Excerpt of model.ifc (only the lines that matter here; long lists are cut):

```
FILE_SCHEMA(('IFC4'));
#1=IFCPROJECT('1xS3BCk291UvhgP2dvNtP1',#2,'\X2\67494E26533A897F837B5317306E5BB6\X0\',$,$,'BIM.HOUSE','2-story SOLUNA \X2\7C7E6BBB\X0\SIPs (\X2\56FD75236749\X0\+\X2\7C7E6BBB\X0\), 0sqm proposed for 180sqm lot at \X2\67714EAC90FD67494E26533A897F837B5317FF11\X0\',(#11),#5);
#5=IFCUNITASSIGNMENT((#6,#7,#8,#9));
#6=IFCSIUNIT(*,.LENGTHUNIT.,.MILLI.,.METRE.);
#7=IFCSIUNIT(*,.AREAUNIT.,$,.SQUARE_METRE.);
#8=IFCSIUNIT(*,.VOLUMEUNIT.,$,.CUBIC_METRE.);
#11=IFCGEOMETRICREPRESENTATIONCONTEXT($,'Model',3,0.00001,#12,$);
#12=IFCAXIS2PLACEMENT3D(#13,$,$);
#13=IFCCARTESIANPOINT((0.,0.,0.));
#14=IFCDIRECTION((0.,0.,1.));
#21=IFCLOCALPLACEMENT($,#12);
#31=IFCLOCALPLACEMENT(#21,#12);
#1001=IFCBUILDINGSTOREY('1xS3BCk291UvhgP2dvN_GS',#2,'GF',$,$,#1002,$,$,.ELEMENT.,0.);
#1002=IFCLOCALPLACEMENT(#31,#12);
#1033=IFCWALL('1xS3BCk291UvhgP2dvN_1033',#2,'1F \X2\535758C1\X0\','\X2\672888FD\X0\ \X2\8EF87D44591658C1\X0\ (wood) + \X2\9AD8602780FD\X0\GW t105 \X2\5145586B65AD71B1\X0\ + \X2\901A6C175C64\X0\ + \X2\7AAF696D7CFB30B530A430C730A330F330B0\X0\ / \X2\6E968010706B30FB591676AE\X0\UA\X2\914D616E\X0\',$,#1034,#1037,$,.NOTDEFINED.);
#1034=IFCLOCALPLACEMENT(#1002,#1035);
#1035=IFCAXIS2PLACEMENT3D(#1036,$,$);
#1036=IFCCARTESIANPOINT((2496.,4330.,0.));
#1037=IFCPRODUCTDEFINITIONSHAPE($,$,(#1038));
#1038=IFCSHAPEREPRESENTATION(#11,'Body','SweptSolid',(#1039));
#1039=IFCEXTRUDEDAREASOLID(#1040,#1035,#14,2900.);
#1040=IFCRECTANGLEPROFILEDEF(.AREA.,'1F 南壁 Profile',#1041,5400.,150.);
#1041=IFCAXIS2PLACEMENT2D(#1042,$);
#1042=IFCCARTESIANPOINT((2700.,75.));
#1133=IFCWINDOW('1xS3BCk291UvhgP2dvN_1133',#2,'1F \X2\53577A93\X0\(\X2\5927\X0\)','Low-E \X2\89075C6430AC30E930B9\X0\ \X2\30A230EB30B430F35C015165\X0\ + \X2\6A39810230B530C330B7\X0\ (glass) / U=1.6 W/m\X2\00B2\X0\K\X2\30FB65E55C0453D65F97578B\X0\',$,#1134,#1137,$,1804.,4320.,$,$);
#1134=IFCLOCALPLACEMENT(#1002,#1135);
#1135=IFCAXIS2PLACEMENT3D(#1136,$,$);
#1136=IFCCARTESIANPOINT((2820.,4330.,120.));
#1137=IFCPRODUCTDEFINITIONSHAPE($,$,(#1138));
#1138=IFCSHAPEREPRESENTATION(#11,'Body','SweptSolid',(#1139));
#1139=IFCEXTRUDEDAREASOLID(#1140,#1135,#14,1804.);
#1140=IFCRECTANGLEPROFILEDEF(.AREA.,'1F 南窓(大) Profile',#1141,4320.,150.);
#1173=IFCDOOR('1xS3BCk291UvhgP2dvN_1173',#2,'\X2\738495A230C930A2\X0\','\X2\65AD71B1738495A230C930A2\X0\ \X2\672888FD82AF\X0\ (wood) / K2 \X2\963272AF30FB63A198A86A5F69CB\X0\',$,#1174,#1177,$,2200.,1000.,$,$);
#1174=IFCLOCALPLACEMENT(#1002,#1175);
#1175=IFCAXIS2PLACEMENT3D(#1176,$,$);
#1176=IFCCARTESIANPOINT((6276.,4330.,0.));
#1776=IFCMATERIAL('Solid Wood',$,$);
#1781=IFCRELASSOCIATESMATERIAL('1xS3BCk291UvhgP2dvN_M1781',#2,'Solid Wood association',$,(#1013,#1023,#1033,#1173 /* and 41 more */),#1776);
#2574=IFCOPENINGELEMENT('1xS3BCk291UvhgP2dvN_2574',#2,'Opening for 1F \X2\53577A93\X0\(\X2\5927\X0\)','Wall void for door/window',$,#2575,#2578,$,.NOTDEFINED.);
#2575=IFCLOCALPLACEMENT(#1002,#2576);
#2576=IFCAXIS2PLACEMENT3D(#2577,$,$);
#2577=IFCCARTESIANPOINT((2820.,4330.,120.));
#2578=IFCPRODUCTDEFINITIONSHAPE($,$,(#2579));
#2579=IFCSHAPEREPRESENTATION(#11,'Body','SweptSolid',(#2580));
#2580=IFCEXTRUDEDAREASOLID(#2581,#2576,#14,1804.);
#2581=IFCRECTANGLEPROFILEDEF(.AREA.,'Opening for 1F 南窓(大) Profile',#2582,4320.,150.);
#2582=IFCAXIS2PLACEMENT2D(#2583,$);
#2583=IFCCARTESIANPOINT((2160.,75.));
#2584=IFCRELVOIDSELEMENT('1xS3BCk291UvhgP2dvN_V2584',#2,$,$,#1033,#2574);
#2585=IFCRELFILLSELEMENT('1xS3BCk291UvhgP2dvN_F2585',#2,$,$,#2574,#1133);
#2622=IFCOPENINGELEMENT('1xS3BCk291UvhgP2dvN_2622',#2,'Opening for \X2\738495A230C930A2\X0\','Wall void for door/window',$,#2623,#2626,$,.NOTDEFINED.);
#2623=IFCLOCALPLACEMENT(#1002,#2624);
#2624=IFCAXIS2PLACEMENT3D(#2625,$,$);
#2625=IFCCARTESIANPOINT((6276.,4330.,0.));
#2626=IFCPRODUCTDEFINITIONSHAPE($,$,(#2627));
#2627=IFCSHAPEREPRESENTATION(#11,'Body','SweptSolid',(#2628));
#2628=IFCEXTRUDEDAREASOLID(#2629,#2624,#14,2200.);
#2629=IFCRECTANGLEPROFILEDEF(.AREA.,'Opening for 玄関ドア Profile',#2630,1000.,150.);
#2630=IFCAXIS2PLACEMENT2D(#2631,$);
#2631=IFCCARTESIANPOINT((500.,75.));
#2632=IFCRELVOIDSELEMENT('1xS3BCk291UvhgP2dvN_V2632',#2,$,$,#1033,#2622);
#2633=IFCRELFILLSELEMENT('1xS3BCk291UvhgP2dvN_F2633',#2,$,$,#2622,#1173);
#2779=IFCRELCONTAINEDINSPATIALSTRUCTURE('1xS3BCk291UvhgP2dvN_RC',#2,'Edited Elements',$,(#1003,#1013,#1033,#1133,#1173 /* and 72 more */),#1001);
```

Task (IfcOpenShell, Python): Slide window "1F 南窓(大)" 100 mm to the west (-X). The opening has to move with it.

```python
import ifcopenshell
import ifcopenshell.api.geometry
import ifcopenshell.util.placement
import ifcopenshell.util.unit

model = ifcopenshell.open("model.ifc")
unit_scale = ifcopenshell.util.unit.calculate_unit_scale(model)

window = model.by_id(1133)
opening = window.FillsVoids[0].RelatingOpeningElement
wall = opening.VoidsElements[0].RelatingBuildingElement

wall_matrix = ifcopenshell.util.placement.get_local_placement(wall.ObjectPlacement)
shift = wall_matrix[:3, 0] * -0.1 / unit_scale
before = ifcopenshell.util.placement.get_local_placement(window.ObjectPlacement)[:3, 3].copy()

# The window is not placed relative to its opening, so move both.
for product in (opening, window):
    matrix = ifcopenshell.util.placement.get_local_placement(product.ObjectPlacement)
    matrix[:3, 3] += shift
    ifcopenshell.api.geometry.edit_object_placement(model, product=product, matrix=matrix, is_si=False)

after = ifcopenshell.util.placement.get_local_placement(window.ObjectPlacement)[:3, 3]
print("window moved by", (after - before).round(3) + 0.0)

model.write("model_updated.ifc")
```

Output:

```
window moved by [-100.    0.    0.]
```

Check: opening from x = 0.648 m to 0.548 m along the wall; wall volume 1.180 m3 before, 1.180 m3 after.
